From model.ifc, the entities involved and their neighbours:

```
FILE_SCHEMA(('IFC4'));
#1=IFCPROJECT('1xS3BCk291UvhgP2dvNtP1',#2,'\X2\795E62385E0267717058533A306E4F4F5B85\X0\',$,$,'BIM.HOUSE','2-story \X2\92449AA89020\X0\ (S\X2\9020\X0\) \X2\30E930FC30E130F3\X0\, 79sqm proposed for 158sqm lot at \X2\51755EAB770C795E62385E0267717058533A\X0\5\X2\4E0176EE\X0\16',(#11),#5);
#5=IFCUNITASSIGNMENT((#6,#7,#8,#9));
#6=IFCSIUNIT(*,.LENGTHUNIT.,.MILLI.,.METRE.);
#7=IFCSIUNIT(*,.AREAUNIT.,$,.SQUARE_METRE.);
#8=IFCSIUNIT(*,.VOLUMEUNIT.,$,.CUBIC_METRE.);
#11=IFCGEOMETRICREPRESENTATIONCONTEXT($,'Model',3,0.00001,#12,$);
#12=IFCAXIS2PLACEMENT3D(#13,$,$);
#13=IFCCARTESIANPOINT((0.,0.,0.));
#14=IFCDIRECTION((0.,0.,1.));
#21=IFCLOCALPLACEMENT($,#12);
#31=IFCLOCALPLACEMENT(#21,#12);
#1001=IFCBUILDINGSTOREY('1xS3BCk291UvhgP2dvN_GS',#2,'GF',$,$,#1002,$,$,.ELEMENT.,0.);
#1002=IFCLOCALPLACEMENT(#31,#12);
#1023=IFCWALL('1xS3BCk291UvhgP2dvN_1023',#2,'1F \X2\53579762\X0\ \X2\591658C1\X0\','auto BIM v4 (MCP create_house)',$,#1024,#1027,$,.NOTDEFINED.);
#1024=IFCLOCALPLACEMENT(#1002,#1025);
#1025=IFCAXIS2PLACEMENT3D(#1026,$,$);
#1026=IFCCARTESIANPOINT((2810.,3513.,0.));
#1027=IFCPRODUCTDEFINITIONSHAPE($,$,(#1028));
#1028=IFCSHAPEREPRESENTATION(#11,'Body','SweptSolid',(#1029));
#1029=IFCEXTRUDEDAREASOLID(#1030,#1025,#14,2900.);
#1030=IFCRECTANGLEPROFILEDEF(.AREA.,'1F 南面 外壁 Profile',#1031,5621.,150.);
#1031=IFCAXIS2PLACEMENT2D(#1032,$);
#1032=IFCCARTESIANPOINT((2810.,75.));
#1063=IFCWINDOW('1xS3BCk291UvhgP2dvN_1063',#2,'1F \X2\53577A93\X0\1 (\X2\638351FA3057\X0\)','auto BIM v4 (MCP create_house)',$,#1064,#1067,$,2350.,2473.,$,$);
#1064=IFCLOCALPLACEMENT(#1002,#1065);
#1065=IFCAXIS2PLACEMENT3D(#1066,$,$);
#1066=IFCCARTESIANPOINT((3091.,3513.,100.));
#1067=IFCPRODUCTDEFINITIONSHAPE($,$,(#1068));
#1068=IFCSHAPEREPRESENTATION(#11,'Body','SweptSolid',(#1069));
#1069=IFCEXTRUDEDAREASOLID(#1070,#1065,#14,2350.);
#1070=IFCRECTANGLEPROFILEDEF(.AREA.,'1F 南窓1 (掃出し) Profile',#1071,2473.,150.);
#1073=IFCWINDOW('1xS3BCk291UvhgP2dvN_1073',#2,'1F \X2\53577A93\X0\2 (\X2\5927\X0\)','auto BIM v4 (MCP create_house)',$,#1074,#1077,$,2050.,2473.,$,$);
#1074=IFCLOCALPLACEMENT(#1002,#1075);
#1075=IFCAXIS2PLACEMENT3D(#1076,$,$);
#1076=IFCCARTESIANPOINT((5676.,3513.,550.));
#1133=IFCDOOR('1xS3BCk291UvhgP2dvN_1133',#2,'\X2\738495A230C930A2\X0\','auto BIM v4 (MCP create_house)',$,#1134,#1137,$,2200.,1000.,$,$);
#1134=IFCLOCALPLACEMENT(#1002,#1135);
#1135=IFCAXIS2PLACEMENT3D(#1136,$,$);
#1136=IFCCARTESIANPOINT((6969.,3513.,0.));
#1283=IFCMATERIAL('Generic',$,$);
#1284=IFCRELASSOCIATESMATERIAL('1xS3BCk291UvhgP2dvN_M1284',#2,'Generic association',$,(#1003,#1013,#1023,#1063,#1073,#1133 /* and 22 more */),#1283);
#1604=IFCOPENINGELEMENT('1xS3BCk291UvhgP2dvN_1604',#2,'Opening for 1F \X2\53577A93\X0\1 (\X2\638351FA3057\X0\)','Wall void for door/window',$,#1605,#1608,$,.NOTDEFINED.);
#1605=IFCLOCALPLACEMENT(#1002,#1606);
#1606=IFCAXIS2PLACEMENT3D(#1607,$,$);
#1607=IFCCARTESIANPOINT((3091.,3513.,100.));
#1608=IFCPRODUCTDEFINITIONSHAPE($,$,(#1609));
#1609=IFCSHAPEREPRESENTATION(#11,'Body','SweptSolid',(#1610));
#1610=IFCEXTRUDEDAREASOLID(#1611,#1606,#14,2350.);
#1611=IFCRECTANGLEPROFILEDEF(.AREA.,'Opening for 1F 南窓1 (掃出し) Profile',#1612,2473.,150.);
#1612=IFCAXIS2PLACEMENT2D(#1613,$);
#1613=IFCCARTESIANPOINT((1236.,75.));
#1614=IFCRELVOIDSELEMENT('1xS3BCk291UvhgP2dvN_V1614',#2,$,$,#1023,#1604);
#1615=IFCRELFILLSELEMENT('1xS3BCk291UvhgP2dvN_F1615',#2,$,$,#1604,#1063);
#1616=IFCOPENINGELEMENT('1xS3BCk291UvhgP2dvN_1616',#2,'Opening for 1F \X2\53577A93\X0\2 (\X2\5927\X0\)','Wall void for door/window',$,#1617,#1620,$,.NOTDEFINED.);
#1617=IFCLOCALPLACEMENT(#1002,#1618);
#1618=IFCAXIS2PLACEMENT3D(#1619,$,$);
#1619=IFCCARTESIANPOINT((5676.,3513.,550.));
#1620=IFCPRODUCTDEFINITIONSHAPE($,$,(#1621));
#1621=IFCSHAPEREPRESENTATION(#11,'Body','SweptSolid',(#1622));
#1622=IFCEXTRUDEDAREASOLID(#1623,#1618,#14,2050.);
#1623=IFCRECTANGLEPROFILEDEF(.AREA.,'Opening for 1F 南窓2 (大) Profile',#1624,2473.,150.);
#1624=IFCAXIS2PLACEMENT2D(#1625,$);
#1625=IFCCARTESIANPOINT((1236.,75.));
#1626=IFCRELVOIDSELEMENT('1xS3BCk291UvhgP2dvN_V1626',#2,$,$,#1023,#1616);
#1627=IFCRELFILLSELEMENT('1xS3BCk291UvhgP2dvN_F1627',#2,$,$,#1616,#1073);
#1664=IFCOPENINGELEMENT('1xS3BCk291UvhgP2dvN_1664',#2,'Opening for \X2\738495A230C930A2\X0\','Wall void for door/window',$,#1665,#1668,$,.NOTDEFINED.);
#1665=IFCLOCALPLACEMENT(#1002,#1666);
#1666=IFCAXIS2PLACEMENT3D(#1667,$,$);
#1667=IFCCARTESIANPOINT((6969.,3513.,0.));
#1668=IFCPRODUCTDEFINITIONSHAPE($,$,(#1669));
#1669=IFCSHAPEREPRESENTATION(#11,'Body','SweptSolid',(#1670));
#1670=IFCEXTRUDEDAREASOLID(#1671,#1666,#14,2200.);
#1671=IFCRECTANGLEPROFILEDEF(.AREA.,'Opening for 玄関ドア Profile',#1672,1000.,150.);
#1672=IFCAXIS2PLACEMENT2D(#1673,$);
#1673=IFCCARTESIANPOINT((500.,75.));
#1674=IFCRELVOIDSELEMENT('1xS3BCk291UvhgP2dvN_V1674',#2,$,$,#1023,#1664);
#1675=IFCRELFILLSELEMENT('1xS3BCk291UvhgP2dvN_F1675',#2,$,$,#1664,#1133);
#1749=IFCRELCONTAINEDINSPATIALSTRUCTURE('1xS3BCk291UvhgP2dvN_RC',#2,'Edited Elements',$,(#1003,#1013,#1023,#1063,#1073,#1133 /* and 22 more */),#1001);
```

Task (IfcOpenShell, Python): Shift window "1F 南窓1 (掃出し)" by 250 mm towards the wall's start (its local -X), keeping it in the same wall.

```python
import ifcopenshell
import ifcopenshell.api.geometry
import ifcopenshell.util.placement

model = ifcopenshell.open("model.ifc")

window = model.by_id(1063)
opening = window.FillsVoids[0].RelatingOpeningElement
wall = opening.VoidsElements[0].RelatingBuildingElement

wall_matrix = ifcopenshell.util.placement.get_local_placement(wall.ObjectPlacement)
shift = wall_matrix[:3, 0] * -250.0
before = ifcopenshell.util.placement.get_local_placement(window.ObjectPlacement)[:3, 3].copy()

# The window is not placed relative to its opening, so move both.
for product in (opening, window):
    matrix = ifcopenshell.util.placement.get_local_placement(product.ObjectPlacement)
    matrix[:3, 3] += shift
    ifcopenshell.api.geometry.edit_object_placement(model, product=product, matrix=matrix, is_si=False)

after = ifcopenshell.util.placement.get_local_placement(window.ObjectPlacement)[:3, 3]
print("window moved by", (after - before).round(3) + 0.0)

model.write("model_edited.ifc")
```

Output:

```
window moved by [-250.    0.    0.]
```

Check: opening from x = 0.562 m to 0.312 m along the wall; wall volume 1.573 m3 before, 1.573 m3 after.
